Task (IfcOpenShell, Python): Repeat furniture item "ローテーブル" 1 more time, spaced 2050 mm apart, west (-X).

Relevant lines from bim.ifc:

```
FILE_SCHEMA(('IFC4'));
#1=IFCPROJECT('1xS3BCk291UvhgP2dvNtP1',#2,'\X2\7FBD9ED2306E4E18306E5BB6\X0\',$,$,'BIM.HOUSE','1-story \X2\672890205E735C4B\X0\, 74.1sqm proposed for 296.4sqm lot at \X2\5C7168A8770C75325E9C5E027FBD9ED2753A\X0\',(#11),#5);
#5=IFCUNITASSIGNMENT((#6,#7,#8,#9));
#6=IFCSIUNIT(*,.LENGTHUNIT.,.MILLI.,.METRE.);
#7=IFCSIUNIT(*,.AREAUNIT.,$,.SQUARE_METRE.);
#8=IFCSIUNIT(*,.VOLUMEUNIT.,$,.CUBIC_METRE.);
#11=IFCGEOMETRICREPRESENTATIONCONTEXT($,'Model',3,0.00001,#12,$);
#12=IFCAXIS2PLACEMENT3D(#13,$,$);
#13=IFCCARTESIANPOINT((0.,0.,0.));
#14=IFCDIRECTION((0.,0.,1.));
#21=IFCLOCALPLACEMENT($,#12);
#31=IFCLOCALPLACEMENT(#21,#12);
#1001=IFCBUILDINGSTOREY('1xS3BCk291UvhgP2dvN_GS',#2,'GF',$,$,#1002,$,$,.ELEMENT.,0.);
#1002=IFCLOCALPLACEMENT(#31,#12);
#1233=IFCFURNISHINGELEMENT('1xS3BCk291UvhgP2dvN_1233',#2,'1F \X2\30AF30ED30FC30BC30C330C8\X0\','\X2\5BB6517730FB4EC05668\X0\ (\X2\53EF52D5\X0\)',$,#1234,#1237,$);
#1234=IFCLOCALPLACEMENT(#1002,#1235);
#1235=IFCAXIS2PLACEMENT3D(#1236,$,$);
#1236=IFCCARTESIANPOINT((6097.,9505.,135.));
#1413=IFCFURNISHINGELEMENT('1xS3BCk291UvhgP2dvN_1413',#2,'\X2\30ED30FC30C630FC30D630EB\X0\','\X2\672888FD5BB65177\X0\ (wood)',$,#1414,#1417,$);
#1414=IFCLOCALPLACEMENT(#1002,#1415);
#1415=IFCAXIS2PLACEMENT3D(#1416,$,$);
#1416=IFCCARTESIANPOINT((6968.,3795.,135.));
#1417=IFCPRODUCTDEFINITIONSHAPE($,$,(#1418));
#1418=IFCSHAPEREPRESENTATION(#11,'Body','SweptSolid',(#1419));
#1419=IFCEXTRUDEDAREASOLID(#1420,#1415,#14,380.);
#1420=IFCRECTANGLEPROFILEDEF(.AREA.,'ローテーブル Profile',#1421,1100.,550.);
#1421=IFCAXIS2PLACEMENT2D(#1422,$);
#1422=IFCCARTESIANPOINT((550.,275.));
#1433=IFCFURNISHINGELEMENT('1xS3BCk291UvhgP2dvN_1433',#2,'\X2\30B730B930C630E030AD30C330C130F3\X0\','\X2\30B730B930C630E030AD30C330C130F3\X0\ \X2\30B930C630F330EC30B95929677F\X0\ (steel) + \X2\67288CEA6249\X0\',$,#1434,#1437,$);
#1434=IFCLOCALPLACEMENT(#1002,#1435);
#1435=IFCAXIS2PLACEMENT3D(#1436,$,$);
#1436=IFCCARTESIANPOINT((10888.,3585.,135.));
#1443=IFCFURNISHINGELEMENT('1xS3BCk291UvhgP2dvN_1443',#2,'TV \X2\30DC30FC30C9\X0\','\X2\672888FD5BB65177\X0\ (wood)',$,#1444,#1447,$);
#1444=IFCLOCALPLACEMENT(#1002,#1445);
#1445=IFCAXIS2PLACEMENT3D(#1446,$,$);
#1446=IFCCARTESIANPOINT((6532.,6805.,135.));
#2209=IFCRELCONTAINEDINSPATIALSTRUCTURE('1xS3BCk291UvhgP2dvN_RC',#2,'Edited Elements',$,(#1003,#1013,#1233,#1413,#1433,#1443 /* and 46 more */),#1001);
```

```python
import numpy as np
import ifcopenshell
import ifcopenshell.api.geometry
import ifcopenshell.api.root
import ifcopenshell.util.element
import ifcopenshell.util.placement

model = ifcopenshell.open("bim.ifc")


def reuse_history(source, copy):
    """copy_class also copies each property set's owner history, people and application; keep the originals."""
    for rel in copy.IsDefinedBy:
        if rel.is_a("IfcRelDefinesByProperties") and (history := rel.RelatingPropertyDefinition.OwnerHistory):
            rel.RelatingPropertyDefinition.OwnerHistory = source.OwnerHistory
            ifcopenshell.util.element.remove_deep2(model, history)


source = model.by_guid("1xS3BCk291UvhgP2dvN_1413")
base = ifcopenshell.util.placement.get_local_placement(source.ObjectPlacement)
step = np.array([-1.0, 0.0, 0.0]) * 2050.0

for i in range(1, 2):
    copy = ifcopenshell.api.root.copy_class(model, product=source)
    copy.Representation = ifcopenshell.util.element.copy_deep(
        model, source.Representation, exclude=["IfcGeometricRepresentationContext", "IfcRepresentationMap"]
    )
    reuse_history(source, copy)
    matrix = base.copy()
    matrix[:3, 3] += i * step
    print("added at", matrix[:3, 3].round(3) + 0.0)
    ifcopenshell.api.geometry.edit_object_placement(model, product=copy, matrix=matrix, is_si=False)

model.write("bim_updated.ifc")
```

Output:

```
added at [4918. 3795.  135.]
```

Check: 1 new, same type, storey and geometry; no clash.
